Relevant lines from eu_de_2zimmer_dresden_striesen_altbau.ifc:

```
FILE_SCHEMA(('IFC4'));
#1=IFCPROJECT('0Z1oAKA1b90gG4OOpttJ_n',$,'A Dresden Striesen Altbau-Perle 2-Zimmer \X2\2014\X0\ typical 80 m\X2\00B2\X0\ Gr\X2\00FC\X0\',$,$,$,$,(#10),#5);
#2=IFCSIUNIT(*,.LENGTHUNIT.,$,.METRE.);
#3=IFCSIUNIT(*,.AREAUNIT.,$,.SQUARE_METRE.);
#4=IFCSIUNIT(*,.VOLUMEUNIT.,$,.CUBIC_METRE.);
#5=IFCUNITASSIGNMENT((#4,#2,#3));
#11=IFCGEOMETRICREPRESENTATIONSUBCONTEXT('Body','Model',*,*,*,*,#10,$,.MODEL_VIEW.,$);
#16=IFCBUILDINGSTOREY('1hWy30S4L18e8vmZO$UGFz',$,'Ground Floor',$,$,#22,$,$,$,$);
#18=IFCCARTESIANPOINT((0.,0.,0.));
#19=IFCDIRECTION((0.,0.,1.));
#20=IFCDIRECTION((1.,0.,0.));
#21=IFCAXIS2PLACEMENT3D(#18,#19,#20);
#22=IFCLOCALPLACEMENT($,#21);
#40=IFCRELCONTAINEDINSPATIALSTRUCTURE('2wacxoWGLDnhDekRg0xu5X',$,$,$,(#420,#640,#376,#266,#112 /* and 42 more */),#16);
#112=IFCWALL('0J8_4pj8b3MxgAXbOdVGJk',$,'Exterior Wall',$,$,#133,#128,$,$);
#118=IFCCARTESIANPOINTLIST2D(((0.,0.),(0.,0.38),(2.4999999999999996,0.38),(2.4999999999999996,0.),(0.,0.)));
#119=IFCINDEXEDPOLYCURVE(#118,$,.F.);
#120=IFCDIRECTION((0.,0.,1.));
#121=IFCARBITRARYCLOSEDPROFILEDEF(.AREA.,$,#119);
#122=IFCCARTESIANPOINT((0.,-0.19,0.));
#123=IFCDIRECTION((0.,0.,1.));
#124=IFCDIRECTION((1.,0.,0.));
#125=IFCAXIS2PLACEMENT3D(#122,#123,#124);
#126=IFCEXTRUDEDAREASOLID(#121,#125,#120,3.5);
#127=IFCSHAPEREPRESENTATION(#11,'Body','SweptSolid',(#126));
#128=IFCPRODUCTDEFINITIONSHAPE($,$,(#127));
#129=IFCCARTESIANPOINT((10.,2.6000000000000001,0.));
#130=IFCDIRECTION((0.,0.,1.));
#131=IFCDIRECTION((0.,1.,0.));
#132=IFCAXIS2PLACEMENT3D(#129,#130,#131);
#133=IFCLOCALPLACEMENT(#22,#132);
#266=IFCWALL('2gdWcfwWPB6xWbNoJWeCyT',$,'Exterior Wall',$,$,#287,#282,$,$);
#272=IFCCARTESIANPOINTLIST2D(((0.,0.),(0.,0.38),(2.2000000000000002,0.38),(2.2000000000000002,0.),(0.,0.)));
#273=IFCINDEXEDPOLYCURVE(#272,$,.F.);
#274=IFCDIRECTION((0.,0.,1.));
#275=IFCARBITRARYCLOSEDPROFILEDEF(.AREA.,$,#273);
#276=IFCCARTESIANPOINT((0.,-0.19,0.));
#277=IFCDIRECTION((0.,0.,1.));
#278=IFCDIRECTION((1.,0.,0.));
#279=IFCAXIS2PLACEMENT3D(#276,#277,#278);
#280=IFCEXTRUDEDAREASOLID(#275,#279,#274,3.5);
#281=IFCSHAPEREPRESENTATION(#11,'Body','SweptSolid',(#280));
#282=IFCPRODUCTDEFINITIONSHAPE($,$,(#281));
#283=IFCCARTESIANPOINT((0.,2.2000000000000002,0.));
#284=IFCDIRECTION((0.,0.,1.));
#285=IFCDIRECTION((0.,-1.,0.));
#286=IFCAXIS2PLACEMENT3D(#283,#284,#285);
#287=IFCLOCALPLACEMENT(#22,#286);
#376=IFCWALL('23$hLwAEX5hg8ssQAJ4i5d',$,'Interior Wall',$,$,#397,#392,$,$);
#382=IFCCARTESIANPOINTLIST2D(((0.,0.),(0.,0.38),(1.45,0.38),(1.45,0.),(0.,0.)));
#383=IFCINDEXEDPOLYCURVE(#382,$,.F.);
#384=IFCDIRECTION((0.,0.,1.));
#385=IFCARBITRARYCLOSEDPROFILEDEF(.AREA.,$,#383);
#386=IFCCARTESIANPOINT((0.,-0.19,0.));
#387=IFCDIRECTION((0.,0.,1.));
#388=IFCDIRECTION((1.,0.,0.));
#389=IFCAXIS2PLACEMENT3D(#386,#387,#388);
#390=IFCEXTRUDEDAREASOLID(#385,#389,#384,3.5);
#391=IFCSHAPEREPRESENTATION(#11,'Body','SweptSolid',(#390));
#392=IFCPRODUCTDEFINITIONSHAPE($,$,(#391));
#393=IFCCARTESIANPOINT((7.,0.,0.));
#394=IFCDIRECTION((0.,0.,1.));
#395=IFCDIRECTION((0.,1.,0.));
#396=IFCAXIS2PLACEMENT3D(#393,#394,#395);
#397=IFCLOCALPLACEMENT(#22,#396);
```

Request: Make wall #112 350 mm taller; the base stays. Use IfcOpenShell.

```python
import ifcopenshell
import ifcopenshell.geom
import ifcopenshell.util.representation
import ifcopenshell.util.shape
import ifcopenshell.util.unit

model = ifcopenshell.open("eu_de_2zimmer_dresden_striesen_altbau.ifc")
unit_scale = ifcopenshell.util.unit.calculate_unit_scale(model)
settings = ifcopenshell.geom.settings()


def volume(element):
    """Net volume in cubic metres, openings subtracted."""
    shape = ifcopenshell.geom.create_shape(settings, element)
    return ifcopenshell.util.shape.get_volume(shape.geometry)


wall = model.by_guid("0J8_4pj8b3MxgAXbOdVGJk")
before = volume(wall)

body = ifcopenshell.util.representation.get_representation(wall, "Model", "Body")
solid = body.Items[0]
old_height = solid.Depth
solid.Depth += 0.35 / unit_scale
after = volume(wall)

print(f"height {old_height:g} -> {solid.Depth:g}, volume {before:.3f} -> {after:.3f} m3")

model.write("eu_de_2zimmer_dresden_striesen_altbau-out.ifc")
```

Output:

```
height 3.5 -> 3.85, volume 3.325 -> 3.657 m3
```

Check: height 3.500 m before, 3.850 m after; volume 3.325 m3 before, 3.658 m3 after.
